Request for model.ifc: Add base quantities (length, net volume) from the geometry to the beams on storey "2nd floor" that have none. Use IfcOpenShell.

First a look at what the model holds.

```python
import ifcopenshell
import ifcopenshell.util.element
import ifcopenshell.util.unit

model = ifcopenshell.open("model.ifc")
print(model.schema)
for unit_type in ("LENGTHUNIT", "AREAUNIT", "VOLUMEUNIT"):
    print(unit_type, ifcopenshell.util.unit.calculate_unit_scale(model, unit_type))
storey = next(s for s in model.by_type("IfcBuildingStorey") if s.Name == "2nd floor")
beams = [e for e in ifcopenshell.util.element.get_decomposition(storey) if e.is_a("IfcBeam")]
for e in sorted(beams, key=lambda e: e.id()):
    print(e.id(), e.is_a(), e.Name, list(ifcopenshell.util.element.get_psets(e, qtos_only=True)), sep=" | ")
```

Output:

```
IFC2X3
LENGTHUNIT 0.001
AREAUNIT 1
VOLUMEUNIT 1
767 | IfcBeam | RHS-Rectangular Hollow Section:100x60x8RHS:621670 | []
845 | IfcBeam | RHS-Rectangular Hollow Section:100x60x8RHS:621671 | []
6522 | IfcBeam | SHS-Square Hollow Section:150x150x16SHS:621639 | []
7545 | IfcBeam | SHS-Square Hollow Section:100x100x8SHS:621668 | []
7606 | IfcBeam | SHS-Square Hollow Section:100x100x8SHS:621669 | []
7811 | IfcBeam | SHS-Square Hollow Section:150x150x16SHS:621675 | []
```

```python
import ifcopenshell
import ifcopenshell.api.pset
import ifcopenshell.geom
import ifcopenshell.util.element
import ifcopenshell.util.shape
import ifcopenshell.util.unit

model = ifcopenshell.open("model.ifc")
unit_scale = ifcopenshell.util.unit.calculate_unit_scale(model)
volume_scale = ifcopenshell.util.unit.calculate_unit_scale(model, "VOLUMEUNIT")
settings = ifcopenshell.geom.settings()

storey = next(s for s in model.by_type("IfcBuildingStorey") if s.Name == "2nd floor")
beams = [e for e in ifcopenshell.util.element.get_decomposition(storey) if e.is_a("IfcBeam")]

for e in sorted(beams, key=lambda e: e.id()):
    if ifcopenshell.util.element.get_psets(e, qtos_only=True, should_inherit=False):
        continue
    # Geometry comes back in metres, in the element's own axes.
    shape = ifcopenshell.geom.create_shape(settings, e)
    values = {
        "Length": ifcopenshell.util.shape.get_max_xyz(shape.geometry) / unit_scale,
        "NetVolume": ifcopenshell.util.shape.get_volume(shape.geometry) / volume_scale,
    }
    qto = ifcopenshell.api.pset.add_qto(model, product=e, name="BaseQuantities")
    ifcopenshell.api.pset.edit_qto(model, qto=qto, properties=values)
    print(e.id(), {k: round(v, 3) for k, v in values.items()})

model.write("model_edited.ifc")
```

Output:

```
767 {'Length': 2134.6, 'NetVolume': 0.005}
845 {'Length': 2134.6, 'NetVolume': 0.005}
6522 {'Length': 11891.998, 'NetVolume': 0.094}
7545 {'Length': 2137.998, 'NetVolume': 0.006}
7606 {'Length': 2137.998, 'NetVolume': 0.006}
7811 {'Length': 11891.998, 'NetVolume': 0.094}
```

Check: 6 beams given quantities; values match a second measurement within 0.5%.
